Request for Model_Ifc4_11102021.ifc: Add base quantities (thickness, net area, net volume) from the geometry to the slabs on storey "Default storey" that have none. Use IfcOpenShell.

First a look at what the model holds.

```python
import ifcopenshell
import ifcopenshell.util.element
import ifcopenshell.util.unit

model = ifcopenshell.open("Model_Ifc4_11102021.ifc")
print(model.schema)
for unit_type in ("LENGTHUNIT", "AREAUNIT", "VOLUMEUNIT"):
    print(unit_type, ifcopenshell.util.unit.calculate_unit_scale(model, unit_type))
storey = next(s for s in model.by_type("IfcBuildingStorey") if s.Name == "Default storey")
slabs = [e for e in ifcopenshell.util.element.get_decomposition(storey) if e.is_a("IfcSlab")]
for e in sorted(slabs, key=lambda e: e.id()):
    print(e.id(), e.is_a(), e.Name, list(ifcopenshell.util.element.get_psets(e, qtos_only=True)), sep=" | ")
```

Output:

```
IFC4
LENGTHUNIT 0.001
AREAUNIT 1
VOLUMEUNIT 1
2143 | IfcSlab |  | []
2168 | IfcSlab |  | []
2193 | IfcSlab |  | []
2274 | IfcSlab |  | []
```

```python
import ifcopenshell
import ifcopenshell.api.pset
import ifcopenshell.geom
import ifcopenshell.util.element
import ifcopenshell.util.shape
import ifcopenshell.util.unit

model = ifcopenshell.open("Model_Ifc4_11102021.ifc")
unit_scale = ifcopenshell.util.unit.calculate_unit_scale(model)
area_scale = ifcopenshell.util.unit.calculate_unit_scale(model, "AREAUNIT")
volume_scale = ifcopenshell.util.unit.calculate_unit_scale(model, "VOLUMEUNIT")
settings = ifcopenshell.geom.settings()

storey = next(s for s in model.by_type("IfcBuildingStorey") if s.Name == "Default storey")
slabs = [e for e in ifcopenshell.util.element.get_decomposition(storey) if e.is_a("IfcSlab")]

for e in sorted(slabs, key=lambda e: e.id()):
    if ifcopenshell.util.element.get_psets(e, qtos_only=True, should_inherit=False):
        continue
    # Geometry comes back in metres, in the element's own axes.
    shape = ifcopenshell.geom.create_shape(settings, e)
    values = {
        "Width": ifcopenshell.util.shape.get_z(shape.geometry) / unit_scale,
        "NetArea": ifcopenshell.util.shape.get_footprint_area(shape.geometry) / area_scale,
        "NetVolume": ifcopenshell.util.shape.get_volume(shape.geometry) / volume_scale,
    }
    qto = ifcopenshell.api.pset.add_qto(model, product=e, name="Qto_SlabBaseQuantities")
    ifcopenshell.api.pset.edit_qto(model, qto=qto, properties=values)
    print(e.id(), {k: round(v, 3) for k, v in values.items()})

model.write("Model_Ifc4_11102021_v2.ifc")
```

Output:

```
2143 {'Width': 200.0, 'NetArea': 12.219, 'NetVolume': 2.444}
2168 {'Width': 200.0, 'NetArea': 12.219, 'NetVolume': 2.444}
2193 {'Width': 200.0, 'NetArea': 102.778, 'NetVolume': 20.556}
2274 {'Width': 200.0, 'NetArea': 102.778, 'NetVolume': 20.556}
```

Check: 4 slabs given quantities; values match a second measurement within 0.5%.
